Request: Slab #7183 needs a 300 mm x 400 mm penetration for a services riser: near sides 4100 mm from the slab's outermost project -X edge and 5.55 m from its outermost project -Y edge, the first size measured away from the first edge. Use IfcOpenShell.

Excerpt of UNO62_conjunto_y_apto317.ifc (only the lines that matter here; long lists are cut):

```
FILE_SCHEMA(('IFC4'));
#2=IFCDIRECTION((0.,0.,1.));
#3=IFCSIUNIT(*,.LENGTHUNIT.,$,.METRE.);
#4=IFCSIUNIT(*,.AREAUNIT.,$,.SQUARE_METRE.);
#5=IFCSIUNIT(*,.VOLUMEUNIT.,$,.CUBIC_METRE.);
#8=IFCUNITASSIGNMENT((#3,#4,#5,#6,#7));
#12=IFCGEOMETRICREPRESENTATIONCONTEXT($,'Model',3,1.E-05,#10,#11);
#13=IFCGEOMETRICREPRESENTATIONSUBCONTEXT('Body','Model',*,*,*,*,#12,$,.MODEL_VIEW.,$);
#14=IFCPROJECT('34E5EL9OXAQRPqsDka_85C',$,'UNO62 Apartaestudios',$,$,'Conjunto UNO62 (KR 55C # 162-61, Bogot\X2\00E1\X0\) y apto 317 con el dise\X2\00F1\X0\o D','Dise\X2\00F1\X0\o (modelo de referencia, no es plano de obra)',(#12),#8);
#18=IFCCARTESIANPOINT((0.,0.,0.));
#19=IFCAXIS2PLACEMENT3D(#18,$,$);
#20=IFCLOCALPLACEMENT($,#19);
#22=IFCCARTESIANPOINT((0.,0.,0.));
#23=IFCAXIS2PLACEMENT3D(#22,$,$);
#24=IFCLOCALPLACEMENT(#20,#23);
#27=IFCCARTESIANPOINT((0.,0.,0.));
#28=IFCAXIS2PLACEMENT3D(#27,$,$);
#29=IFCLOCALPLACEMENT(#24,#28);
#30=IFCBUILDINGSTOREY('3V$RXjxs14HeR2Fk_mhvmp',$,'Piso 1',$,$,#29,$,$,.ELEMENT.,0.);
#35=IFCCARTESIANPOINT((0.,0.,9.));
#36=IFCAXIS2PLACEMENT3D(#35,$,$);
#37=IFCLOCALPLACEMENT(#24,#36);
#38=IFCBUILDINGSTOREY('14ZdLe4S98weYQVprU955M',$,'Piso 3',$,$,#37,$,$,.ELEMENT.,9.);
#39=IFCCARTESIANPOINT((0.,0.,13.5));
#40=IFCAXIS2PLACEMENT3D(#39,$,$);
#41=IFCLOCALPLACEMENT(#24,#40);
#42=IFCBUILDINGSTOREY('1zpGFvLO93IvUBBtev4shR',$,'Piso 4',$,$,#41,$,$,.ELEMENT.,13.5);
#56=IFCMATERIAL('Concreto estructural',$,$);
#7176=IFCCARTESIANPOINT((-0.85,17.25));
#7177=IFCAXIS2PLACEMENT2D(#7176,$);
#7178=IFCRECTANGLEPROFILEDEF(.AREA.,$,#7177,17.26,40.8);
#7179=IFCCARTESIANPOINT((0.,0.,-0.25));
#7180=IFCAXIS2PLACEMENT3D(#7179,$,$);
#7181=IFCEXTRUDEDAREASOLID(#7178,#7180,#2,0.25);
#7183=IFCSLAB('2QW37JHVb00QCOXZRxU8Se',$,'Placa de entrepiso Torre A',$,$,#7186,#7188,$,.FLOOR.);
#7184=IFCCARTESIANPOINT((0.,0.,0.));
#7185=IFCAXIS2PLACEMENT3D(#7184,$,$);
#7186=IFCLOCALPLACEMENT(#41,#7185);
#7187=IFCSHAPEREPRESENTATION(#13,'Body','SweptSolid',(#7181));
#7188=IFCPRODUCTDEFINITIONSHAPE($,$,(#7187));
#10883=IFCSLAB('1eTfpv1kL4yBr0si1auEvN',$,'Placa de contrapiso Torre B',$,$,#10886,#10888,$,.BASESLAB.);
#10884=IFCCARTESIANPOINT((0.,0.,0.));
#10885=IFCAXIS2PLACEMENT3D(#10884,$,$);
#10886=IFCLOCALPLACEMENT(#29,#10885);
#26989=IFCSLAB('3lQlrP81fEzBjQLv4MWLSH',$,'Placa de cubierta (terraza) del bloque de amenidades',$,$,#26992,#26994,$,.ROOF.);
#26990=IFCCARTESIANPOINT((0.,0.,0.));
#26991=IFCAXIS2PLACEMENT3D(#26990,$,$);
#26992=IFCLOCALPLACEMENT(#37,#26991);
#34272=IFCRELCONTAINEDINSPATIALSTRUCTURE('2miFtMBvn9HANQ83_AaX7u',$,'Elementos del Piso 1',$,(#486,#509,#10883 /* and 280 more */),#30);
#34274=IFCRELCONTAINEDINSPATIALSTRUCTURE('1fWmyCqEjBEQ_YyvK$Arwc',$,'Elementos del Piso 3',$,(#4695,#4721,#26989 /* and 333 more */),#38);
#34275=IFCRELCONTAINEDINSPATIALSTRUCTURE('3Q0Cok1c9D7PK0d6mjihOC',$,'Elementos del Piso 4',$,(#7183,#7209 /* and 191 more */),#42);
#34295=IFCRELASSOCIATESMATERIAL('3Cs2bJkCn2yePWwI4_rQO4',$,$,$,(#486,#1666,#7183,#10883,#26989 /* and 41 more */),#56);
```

```python
import numpy as np
import ifcopenshell
import ifcopenshell.api.feature
import ifcopenshell.api.geometry
import ifcopenshell.api.root
import ifcopenshell.geom
import ifcopenshell.util.placement
import ifcopenshell.util.representation
import ifcopenshell.util.shape
import ifcopenshell.util.unit

model = ifcopenshell.open("UNO62_conjunto_y_apto317.ifc")
unit_scale = ifcopenshell.util.unit.calculate_unit_scale(model)
settings = ifcopenshell.geom.settings()


def volume(element):
    """Net volume in cubic metres, openings subtracted."""
    shape = ifcopenshell.geom.create_shape(settings, element)
    return ifcopenshell.util.shape.get_volume(shape.geometry)


slab = model.by_id(7183)
before = volume(slab)

# Extent in the slab's own axes, in metres. The edges named are its -X and -Y sides.
slab_shape = ifcopenshell.geom.create_shape(settings, slab)
vertices = ifcopenshell.util.shape.get_vertices(slab_shape.geometry)
x_min, y_min, bottom = vertices.min(axis=0)
top = vertices[:, 2].max()

opening = ifcopenshell.api.root.create_entity(model, ifc_class="IfcOpeningElement", name="Services riser opening", predefined_type="OPENING")
context = ifcopenshell.util.representation.get_context(model, "Model", "Body", "MODEL_VIEW")
width, depth = 0.3, 0.4
outline = [(0.0, 0.0), (width, 0.0), (width, depth), (0.0, depth), (0.0, 0.0)]
# Overshoot both faces by 50 mm so the cut is clean.
shape = ifcopenshell.api.geometry.add_slab_representation(
    model, context=context, depth=top - bottom + 0.1, polyline=outline
)
ifcopenshell.api.geometry.assign_representation(model, product=opening, representation=shape)

matrix = ifcopenshell.util.placement.get_local_placement(slab.ObjectPlacement)
matrix[:, 3] = matrix @ np.append(np.array([x_min + 4.1, y_min + 5.55, bottom - 0.05]) / unit_scale, 1.0)
ifcopenshell.api.geometry.edit_object_placement(model, product=opening, matrix=matrix, is_si=False)
ifcopenshell.api.feature.add_feature(model, feature=opening, element=slab)

after = volume(slab)

print(f"slab volume {before:.3f} -> {after:.3f} m3")

model.write("UNO62_conjunto_y_apto317_updated.ifc")
```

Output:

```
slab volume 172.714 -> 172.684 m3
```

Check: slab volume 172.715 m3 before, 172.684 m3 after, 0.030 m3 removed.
